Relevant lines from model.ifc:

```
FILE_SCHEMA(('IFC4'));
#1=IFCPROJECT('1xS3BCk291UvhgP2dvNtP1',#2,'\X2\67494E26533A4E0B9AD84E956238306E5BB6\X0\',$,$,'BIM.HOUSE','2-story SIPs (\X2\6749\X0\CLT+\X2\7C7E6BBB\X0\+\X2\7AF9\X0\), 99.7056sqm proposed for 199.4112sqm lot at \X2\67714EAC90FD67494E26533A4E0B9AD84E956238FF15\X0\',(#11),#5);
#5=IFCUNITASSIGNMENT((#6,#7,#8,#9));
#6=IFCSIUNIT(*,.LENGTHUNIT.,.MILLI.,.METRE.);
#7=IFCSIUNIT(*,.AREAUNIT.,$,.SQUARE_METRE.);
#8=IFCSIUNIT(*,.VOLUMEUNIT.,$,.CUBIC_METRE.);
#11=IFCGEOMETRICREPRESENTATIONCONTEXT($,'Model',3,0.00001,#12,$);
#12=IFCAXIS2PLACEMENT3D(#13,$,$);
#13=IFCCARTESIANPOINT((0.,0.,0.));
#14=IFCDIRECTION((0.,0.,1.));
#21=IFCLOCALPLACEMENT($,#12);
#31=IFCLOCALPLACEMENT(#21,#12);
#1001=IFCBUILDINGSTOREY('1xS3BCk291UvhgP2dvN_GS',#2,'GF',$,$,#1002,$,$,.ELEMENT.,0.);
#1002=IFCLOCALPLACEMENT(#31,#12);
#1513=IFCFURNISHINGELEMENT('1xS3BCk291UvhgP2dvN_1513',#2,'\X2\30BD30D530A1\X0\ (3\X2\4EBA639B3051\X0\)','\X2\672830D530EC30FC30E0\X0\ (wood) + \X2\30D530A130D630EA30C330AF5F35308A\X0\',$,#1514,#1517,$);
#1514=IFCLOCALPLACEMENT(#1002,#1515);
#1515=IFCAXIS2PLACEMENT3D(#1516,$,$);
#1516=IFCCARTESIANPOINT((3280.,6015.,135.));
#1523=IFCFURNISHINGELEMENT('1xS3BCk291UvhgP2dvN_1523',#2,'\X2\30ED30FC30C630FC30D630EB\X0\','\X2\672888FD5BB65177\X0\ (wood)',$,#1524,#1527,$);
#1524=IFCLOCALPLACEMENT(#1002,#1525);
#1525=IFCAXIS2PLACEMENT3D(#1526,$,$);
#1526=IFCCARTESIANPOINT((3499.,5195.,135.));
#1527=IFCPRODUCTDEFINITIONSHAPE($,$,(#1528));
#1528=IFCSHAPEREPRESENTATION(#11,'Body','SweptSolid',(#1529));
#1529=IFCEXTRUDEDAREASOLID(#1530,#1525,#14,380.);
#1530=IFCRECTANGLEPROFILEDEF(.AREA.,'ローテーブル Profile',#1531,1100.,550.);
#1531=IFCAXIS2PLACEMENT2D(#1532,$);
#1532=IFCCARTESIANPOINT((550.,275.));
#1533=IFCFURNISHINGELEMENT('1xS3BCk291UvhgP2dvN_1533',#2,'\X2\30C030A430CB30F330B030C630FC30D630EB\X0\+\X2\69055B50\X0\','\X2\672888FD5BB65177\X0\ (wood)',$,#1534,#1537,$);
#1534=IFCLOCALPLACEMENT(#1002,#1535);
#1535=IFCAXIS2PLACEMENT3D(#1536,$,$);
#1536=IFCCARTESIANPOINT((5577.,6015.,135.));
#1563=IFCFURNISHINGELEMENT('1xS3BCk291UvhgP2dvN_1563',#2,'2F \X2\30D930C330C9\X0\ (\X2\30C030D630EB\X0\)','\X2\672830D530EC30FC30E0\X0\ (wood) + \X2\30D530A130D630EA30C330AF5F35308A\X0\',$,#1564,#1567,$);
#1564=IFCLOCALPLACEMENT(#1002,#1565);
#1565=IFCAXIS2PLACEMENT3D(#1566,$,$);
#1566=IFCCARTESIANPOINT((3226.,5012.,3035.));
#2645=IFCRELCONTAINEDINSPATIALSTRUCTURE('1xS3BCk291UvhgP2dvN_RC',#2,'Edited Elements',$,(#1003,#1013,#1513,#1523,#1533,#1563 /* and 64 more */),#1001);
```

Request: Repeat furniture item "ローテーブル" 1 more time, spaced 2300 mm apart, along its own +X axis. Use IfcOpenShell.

```python
import ifcopenshell
import ifcopenshell.api.geometry
import ifcopenshell.api.root
import ifcopenshell.util.element
import ifcopenshell.util.placement
import ifcopenshell.util.unit

model = ifcopenshell.open("model.ifc")
unit_scale = ifcopenshell.util.unit.calculate_unit_scale(model)


def reuse_history(source, copy):
    """copy_class also copies each property set's owner history, people and application; keep the originals."""
    for rel in copy.IsDefinedBy:
        if rel.is_a("IfcRelDefinesByProperties") and (history := rel.RelatingPropertyDefinition.OwnerHistory):
            rel.RelatingPropertyDefinition.OwnerHistory = source.OwnerHistory
            ifcopenshell.util.element.remove_deep2(model, history)


source = model.by_guid("1xS3BCk291UvhgP2dvN_1523")
base = ifcopenshell.util.placement.get_local_placement(source.ObjectPlacement)
step = base[:3, 0] * 2.3 / unit_scale

for i in range(1, 2):
    copy = ifcopenshell.api.root.copy_class(model, product=source)
    copy.Representation = ifcopenshell.util.element.copy_deep(
        model, source.Representation, exclude=["IfcGeometricRepresentationContext", "IfcRepresentationMap"]
    )
    reuse_history(source, copy)
    matrix = base.copy()
    matrix[:3, 3] += i * step
    print("added at", matrix[:3, 3].round(3) + 0.0)
    ifcopenshell.api.geometry.edit_object_placement(model, product=copy, matrix=matrix, is_si=False)

model.write("model_edited.ifc")
```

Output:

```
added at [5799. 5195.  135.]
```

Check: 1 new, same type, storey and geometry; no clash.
